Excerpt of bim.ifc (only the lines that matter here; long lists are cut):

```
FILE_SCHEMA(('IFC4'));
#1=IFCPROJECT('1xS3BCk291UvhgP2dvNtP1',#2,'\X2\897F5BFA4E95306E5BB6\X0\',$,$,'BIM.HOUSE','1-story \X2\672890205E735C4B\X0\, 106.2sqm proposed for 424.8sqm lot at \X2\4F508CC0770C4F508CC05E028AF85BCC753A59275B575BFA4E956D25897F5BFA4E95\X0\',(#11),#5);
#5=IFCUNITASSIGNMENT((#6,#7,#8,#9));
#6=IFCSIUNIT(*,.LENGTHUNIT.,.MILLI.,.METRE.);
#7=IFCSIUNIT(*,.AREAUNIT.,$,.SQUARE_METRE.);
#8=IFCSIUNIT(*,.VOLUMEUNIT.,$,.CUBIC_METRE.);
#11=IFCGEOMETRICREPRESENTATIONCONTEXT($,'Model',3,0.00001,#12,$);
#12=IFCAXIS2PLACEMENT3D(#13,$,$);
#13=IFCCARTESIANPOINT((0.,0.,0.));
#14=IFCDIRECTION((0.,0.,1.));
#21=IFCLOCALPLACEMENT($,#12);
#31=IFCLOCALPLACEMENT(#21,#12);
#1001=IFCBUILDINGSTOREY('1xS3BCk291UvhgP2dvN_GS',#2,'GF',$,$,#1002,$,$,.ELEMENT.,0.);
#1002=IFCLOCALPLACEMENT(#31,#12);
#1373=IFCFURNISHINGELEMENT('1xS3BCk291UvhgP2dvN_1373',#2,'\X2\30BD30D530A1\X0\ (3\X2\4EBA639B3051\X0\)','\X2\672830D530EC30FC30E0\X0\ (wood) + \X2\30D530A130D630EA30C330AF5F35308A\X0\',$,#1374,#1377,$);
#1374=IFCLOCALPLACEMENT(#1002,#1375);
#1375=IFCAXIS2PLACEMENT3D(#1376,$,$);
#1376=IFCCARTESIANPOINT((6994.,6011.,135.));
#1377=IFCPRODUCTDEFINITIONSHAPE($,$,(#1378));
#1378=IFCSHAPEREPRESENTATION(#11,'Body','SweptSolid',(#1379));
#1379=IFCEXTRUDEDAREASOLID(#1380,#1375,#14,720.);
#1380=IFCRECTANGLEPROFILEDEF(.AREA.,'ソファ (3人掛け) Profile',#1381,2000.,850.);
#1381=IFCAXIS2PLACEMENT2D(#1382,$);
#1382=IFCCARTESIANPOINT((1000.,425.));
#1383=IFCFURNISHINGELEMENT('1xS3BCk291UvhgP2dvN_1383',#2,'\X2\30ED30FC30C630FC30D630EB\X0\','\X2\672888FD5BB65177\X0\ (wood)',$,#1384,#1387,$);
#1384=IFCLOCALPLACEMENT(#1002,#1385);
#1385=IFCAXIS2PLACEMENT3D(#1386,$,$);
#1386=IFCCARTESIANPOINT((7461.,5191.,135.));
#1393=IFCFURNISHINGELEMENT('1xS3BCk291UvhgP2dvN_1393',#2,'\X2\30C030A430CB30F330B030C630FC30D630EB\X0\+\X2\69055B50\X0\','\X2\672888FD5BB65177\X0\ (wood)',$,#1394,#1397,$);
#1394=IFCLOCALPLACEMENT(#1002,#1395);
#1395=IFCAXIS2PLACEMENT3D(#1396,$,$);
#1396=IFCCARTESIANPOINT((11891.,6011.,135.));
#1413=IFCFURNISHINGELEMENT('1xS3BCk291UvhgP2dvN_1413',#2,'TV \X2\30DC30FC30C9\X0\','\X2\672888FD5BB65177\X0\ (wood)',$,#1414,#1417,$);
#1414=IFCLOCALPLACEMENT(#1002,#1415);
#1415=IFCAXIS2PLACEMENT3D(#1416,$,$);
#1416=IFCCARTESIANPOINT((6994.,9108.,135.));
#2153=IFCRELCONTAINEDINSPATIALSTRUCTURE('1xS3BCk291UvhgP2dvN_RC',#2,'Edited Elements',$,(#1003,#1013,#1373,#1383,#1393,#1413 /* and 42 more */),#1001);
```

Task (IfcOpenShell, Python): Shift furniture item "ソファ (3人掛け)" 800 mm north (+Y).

```python
import ifcopenshell
import ifcopenshell.api.geometry
import ifcopenshell.util.placement

model = ifcopenshell.open("bim.ifc")

item = model.by_guid("1xS3BCk291UvhgP2dvN_1373")
matrix = ifcopenshell.util.placement.get_local_placement(item.ObjectPlacement)
matrix[1, 3] += 800.0
ifcopenshell.api.geometry.edit_object_placement(model, product=item, matrix=matrix, is_si=False)

print(ifcopenshell.util.placement.get_local_placement(item.ObjectPlacement).round(3) + 0.0)

model.write("bim-out.ifc")
```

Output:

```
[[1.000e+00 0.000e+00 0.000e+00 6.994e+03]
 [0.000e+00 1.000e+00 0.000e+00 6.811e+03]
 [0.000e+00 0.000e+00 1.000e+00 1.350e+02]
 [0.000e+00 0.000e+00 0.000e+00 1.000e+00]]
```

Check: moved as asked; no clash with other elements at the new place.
